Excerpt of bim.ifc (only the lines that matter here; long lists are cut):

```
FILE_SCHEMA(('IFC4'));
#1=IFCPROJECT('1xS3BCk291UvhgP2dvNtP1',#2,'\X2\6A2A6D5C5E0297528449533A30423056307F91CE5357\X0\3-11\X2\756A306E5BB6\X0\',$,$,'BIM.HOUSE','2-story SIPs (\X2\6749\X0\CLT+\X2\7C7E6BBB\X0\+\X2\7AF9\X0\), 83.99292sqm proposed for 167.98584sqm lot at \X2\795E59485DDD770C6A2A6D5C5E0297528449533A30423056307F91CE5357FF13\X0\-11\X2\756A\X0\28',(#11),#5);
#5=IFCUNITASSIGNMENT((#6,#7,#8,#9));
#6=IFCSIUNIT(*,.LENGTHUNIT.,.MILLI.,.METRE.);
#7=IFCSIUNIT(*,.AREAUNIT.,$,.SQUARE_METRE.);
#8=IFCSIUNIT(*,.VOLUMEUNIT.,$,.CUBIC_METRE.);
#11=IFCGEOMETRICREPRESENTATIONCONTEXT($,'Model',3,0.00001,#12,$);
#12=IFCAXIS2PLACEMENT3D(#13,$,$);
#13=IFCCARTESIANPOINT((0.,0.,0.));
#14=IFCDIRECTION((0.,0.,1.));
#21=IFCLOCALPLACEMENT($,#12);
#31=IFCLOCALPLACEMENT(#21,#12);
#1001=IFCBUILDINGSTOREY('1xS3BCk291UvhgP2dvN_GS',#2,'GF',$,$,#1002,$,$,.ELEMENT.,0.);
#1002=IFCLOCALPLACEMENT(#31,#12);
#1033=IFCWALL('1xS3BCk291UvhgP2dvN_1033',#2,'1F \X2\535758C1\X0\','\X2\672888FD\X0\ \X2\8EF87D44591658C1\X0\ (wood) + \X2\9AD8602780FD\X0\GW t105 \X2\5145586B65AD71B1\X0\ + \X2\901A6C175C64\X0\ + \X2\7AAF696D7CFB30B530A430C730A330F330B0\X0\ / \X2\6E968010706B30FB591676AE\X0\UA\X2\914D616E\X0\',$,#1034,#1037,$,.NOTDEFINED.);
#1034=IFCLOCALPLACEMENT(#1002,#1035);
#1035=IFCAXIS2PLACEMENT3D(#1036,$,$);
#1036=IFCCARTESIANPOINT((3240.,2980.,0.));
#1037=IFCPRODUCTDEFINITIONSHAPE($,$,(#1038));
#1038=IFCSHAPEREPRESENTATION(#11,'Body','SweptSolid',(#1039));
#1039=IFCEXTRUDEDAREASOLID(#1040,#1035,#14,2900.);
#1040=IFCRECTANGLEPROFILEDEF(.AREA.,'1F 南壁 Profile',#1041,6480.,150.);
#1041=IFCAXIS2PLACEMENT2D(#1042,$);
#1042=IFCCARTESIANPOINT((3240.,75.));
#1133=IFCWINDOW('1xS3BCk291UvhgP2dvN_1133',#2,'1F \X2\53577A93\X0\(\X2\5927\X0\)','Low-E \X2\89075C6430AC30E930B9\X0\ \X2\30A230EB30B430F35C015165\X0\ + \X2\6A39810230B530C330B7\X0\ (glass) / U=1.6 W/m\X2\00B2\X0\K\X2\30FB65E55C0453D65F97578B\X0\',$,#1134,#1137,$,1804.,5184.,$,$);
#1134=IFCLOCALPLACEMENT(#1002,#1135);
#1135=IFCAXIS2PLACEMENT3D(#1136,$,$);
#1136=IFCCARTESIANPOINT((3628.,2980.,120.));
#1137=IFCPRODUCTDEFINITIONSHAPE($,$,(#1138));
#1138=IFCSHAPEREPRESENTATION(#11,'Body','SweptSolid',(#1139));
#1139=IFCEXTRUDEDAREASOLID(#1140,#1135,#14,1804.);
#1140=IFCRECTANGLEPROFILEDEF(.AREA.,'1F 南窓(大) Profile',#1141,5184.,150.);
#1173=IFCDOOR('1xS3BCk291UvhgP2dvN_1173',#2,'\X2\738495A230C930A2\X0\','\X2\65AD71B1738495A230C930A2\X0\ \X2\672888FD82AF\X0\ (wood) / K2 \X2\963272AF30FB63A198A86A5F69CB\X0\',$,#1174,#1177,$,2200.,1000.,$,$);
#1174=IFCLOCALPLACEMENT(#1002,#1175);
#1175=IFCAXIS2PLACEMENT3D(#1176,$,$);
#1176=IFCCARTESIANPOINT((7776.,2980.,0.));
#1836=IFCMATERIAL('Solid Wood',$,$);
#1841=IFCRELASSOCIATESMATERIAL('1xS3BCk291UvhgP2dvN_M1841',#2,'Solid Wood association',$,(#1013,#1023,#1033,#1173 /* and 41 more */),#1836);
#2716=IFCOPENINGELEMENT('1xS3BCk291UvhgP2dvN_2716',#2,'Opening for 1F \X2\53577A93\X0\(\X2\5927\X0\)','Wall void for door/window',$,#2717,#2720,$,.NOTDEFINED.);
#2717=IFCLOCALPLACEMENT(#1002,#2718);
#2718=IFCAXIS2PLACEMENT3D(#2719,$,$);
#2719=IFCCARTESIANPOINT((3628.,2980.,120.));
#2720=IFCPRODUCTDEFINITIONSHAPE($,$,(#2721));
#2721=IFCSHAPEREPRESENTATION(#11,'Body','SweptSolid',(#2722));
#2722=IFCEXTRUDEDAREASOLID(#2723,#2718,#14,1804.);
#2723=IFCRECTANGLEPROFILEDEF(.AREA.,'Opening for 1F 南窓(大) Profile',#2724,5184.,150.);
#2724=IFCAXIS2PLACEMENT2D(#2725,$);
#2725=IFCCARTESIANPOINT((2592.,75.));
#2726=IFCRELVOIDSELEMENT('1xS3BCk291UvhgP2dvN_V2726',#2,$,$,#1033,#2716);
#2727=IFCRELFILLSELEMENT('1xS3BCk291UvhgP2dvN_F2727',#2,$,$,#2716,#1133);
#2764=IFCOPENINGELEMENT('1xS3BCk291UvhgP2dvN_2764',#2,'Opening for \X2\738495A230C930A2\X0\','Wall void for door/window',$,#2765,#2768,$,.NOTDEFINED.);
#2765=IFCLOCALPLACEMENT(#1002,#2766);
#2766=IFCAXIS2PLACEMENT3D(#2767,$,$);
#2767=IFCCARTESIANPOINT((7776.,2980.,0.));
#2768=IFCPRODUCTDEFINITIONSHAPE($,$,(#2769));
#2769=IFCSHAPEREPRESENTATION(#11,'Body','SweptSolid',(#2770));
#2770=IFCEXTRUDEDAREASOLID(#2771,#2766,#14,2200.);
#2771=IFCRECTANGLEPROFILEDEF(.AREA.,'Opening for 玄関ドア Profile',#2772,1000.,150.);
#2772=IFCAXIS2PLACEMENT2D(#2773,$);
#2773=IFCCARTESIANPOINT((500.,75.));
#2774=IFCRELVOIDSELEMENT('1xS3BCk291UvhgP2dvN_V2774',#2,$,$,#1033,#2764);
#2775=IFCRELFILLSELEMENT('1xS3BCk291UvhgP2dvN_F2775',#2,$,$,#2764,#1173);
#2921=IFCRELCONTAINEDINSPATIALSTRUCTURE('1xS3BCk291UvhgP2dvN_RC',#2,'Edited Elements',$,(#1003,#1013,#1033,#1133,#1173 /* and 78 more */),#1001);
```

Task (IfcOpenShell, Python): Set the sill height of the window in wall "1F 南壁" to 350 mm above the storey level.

```python
import numpy as np
import ifcopenshell
import ifcopenshell.api.geometry
import ifcopenshell.geom
import ifcopenshell.util.element
import ifcopenshell.util.placement
import ifcopenshell.util.shape
import ifcopenshell.util.unit

model = ifcopenshell.open("bim.ifc")
unit_scale = ifcopenshell.util.unit.calculate_unit_scale(model)

window = model.by_id(1133)
opening = window.FillsVoids[0].RelatingOpeningElement
storey = ifcopenshell.util.element.get_container(window, ifc_class="IfcBuildingStorey")
level = ifcopenshell.util.placement.get_local_placement(storey.ObjectPlacement)[2, 3]

# The opening's origin need not be at the sill, so measure its lowest point.
shape = ifcopenshell.geom.create_shape(ifcopenshell.geom.settings(), opening)
bottom = ifcopenshell.util.shape.get_shape_bottom_elevation(shape, shape.geometry) / unit_scale
dz = level + 0.35 / unit_scale - bottom

shift = np.array([0.0, 0.0, dz])
# The window is not placed relative to its opening, so move both.
for product in (opening, window):
    matrix = ifcopenshell.util.placement.get_local_placement(product.ObjectPlacement)
    matrix[:3, 3] += shift
    ifcopenshell.api.geometry.edit_object_placement(model, product=product, matrix=matrix, is_si=False)

print(f"moved by {dz * unit_scale:+.3f} m")

model.write("bim_updated.ifc")
```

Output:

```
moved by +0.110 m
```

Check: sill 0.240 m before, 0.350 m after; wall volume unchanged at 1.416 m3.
